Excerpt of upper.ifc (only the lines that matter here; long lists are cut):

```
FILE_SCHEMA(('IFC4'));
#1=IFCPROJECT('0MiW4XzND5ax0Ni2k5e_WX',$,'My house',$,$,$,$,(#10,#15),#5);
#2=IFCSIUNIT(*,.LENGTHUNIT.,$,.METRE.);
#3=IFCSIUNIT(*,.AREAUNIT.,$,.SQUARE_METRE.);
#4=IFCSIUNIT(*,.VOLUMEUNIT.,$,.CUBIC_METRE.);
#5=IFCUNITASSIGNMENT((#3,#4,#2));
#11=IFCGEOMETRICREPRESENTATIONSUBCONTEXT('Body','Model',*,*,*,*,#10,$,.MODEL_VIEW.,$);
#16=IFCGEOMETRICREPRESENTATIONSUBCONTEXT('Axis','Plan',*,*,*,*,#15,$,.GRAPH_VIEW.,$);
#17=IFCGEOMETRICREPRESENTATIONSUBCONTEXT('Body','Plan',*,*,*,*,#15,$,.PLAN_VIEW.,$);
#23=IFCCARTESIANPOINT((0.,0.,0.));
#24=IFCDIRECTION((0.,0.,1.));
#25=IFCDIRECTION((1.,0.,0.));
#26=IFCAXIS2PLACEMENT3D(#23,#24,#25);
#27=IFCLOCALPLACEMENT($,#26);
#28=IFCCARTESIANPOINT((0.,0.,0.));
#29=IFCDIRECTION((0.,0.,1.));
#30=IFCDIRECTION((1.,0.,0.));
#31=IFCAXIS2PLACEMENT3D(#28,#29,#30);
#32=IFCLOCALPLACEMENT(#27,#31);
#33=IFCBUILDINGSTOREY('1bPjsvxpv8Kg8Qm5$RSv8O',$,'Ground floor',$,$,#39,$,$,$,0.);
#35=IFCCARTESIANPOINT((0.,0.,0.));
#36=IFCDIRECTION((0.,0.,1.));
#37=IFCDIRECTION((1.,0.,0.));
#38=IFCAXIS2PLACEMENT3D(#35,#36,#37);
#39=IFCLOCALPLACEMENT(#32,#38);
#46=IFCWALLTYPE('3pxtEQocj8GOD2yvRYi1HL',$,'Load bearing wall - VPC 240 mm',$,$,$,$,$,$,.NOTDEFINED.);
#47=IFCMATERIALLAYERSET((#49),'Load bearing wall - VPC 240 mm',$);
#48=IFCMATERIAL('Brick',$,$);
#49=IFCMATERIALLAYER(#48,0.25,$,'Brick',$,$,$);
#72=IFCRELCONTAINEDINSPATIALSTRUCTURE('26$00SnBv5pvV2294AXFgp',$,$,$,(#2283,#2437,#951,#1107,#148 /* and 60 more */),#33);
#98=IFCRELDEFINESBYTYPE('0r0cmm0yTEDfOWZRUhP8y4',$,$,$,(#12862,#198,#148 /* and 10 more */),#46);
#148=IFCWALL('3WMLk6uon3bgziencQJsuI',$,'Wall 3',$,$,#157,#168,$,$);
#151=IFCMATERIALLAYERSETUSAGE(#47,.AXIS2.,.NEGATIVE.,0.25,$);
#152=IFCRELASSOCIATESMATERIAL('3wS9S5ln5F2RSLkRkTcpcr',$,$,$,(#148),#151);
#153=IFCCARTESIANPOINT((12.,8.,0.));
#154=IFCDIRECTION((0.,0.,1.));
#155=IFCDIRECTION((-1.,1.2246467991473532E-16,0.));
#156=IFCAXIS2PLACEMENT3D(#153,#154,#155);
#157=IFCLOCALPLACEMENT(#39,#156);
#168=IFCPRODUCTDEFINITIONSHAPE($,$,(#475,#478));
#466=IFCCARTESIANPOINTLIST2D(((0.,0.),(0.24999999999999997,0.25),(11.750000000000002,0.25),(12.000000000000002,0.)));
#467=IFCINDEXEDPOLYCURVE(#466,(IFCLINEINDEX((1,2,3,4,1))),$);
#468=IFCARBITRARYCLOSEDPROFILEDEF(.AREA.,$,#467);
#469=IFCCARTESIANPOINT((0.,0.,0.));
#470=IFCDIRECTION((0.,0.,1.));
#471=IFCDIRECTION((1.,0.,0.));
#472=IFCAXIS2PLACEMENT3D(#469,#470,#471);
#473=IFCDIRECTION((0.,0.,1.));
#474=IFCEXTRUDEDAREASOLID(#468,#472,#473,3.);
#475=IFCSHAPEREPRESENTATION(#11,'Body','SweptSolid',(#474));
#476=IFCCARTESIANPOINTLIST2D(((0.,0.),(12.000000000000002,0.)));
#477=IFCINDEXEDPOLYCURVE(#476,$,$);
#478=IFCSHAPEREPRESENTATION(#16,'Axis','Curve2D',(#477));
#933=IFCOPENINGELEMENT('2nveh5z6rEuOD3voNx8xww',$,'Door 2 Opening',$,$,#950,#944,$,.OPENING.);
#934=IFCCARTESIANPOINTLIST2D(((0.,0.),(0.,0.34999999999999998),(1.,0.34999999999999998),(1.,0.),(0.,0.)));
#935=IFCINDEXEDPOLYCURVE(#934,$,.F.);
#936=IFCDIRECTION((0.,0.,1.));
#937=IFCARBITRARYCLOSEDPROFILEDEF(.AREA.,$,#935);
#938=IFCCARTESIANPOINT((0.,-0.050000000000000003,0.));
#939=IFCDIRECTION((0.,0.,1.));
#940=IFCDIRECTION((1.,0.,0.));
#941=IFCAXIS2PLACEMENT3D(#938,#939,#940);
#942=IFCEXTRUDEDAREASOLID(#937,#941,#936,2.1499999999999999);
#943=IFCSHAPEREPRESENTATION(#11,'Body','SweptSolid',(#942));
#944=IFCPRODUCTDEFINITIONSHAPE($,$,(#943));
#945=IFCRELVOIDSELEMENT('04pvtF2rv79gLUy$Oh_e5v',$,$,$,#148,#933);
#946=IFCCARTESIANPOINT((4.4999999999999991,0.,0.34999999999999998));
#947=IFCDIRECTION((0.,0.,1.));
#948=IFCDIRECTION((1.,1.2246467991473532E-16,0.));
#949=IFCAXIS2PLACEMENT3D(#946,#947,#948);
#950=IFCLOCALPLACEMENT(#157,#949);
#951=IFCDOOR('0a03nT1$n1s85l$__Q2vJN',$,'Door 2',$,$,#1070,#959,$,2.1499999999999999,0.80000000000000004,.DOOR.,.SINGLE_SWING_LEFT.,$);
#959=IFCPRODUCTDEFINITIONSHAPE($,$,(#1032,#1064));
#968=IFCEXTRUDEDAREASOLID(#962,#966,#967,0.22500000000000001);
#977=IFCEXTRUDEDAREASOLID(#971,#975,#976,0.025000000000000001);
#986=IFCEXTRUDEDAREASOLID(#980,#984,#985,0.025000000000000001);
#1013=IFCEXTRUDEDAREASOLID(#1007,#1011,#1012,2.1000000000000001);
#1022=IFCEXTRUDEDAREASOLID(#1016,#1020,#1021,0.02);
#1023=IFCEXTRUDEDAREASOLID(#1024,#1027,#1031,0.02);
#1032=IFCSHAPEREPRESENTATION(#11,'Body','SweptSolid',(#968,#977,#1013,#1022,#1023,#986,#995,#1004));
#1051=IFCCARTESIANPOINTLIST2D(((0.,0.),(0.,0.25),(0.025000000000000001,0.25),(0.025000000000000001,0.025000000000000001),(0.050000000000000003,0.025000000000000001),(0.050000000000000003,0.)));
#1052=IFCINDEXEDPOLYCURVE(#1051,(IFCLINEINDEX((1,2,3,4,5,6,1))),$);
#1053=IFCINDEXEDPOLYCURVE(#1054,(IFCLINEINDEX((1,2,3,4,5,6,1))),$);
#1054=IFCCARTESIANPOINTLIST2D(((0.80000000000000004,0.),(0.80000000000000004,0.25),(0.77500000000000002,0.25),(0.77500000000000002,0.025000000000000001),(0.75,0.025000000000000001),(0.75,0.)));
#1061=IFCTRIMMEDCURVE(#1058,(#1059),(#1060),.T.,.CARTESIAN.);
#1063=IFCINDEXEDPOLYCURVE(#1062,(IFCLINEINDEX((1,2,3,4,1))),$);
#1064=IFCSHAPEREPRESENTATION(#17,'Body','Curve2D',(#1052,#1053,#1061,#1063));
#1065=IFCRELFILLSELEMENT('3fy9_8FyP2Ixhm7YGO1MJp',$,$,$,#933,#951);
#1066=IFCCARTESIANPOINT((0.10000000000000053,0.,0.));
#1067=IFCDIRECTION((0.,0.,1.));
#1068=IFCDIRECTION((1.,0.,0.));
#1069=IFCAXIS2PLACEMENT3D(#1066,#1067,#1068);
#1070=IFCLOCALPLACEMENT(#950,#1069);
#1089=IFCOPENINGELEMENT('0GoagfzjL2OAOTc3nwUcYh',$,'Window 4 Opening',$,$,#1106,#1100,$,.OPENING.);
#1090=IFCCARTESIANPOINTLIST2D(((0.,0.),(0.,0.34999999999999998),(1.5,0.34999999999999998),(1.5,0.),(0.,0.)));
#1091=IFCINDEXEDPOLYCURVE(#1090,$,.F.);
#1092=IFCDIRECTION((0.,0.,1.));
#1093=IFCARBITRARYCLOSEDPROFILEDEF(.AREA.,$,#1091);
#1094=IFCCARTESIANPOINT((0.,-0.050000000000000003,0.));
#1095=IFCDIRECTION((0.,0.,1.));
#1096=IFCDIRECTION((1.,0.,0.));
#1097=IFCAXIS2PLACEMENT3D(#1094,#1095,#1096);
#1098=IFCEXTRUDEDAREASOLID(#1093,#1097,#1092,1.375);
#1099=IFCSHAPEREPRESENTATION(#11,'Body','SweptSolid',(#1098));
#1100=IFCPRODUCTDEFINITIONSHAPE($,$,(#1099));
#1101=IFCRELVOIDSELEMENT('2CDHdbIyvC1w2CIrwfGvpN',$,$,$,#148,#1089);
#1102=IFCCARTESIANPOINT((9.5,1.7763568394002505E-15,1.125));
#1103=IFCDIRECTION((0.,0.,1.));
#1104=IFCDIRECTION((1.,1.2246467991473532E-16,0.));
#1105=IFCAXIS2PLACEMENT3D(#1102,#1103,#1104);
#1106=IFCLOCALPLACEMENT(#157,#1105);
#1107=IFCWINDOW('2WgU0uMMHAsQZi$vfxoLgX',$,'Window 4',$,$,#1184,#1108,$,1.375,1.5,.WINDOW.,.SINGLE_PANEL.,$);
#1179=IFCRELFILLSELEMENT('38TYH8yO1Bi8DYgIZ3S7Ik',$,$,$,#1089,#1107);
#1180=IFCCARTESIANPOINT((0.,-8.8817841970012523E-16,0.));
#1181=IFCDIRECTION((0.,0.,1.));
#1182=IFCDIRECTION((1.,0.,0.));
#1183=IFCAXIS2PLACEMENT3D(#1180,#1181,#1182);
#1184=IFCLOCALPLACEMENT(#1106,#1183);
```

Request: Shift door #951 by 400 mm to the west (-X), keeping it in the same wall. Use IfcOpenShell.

```python
import ifcopenshell
import ifcopenshell.api.geometry
import ifcopenshell.util.placement
import ifcopenshell.util.unit

model = ifcopenshell.open("upper.ifc")
unit_scale = ifcopenshell.util.unit.calculate_unit_scale(model)

door = model.by_guid("0a03nT1$n1s85l$__Q2vJN")
opening = door.FillsVoids[0].RelatingOpeningElement
wall = opening.VoidsElements[0].RelatingBuildingElement

wall_matrix = ifcopenshell.util.placement.get_local_placement(wall.ObjectPlacement)
shift = wall_matrix[:3, 0] * 0.4 / unit_scale
before = ifcopenshell.util.placement.get_local_placement(door.ObjectPlacement)[:3, 3].copy()

# The door is placed relative to its opening, so it follows when the opening moves.
matrix = ifcopenshell.util.placement.get_local_placement(opening.ObjectPlacement)
matrix[:3, 3] += shift
ifcopenshell.api.geometry.edit_object_placement(
    model, product=opening, matrix=matrix, is_si=False, should_transform_children=True
)

after = ifcopenshell.util.placement.get_local_placement(door.ObjectPlacement)[:3, 3]
print("door moved by", (after - before).round(3) + 0.0)

model.write("upper_updated.ifc")
```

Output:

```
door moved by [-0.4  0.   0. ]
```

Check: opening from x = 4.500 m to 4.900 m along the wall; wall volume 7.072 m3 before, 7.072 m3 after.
